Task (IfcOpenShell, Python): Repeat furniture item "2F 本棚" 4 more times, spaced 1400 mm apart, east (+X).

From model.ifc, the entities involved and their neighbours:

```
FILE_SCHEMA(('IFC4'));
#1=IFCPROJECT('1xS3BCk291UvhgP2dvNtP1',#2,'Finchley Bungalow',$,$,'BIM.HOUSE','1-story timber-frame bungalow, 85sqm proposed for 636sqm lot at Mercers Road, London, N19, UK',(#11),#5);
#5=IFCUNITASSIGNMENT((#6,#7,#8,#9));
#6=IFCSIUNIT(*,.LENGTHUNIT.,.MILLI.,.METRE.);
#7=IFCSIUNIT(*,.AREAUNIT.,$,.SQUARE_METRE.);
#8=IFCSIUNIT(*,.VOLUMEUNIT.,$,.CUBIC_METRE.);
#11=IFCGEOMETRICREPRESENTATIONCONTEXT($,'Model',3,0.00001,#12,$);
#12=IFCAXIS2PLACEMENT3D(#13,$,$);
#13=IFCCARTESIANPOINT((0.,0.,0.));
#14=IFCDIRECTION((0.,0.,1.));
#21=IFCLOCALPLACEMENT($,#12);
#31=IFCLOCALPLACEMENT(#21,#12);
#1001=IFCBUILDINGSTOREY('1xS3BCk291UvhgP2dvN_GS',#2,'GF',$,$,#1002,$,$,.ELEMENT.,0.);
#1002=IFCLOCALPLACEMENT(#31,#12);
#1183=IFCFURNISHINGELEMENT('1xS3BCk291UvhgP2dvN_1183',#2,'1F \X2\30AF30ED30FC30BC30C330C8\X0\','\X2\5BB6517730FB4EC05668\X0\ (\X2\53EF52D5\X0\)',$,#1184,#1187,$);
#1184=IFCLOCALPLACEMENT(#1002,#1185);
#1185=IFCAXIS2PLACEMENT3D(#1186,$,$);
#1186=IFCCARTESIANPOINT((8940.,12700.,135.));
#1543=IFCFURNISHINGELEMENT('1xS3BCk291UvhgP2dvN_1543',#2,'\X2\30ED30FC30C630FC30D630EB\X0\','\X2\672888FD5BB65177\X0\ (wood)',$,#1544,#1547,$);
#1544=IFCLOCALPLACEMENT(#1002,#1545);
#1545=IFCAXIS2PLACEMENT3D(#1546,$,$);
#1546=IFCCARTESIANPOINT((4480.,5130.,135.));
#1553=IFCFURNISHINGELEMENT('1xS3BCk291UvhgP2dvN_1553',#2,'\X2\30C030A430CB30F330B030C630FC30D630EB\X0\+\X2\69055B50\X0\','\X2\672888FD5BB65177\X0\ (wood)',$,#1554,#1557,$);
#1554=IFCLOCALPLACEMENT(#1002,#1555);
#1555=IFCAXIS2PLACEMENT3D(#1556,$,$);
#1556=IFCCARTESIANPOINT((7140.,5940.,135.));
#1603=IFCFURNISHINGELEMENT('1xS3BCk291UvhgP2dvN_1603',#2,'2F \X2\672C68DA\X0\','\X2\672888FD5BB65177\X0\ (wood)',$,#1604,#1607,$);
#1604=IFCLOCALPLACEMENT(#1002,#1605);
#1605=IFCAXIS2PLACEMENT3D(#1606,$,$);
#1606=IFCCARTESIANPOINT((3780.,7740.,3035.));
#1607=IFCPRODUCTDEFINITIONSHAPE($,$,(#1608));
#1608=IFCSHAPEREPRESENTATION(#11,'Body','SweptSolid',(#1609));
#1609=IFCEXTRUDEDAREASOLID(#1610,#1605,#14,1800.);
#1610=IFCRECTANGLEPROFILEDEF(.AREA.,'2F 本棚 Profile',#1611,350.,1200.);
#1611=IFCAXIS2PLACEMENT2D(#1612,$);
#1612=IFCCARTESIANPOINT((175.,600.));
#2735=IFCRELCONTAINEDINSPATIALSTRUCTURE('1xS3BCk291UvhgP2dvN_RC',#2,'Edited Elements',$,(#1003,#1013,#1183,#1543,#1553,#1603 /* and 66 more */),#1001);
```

```python
import numpy as np
import ifcopenshell
import ifcopenshell.api.geometry
import ifcopenshell.api.root
import ifcopenshell.util.element
import ifcopenshell.util.placement

model = ifcopenshell.open("model.ifc")


def reuse_history(source, copy):
    """copy_class also copies each property set's owner history, people and application; keep the originals."""
    for rel in copy.IsDefinedBy:
        if rel.is_a("IfcRelDefinesByProperties") and (history := rel.RelatingPropertyDefinition.OwnerHistory):
            rel.RelatingPropertyDefinition.OwnerHistory = source.OwnerHistory
            ifcopenshell.util.element.remove_deep2(model, history)


source = model.by_guid("1xS3BCk291UvhgP2dvN_1603")
base = ifcopenshell.util.placement.get_local_placement(source.ObjectPlacement)
step = np.array([1.0, 0.0, 0.0]) * 1400.0

for i in range(1, 5):
    copy = ifcopenshell.api.root.copy_class(model, product=source)
    copy.Representation = ifcopenshell.util.element.copy_deep(
        model, source.Representation, exclude=["IfcGeometricRepresentationContext", "IfcRepresentationMap"]
    )
    reuse_history(source, copy)
    matrix = base.copy()
    matrix[:3, 3] += i * step
    print("added at", matrix[:3, 3].round(3) + 0.0)
    ifcopenshell.api.geometry.edit_object_placement(model, product=copy, matrix=matrix, is_si=False)

model.write("model-out.ifc")
```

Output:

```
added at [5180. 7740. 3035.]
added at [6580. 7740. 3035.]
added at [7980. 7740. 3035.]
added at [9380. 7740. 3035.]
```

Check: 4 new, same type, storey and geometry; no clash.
